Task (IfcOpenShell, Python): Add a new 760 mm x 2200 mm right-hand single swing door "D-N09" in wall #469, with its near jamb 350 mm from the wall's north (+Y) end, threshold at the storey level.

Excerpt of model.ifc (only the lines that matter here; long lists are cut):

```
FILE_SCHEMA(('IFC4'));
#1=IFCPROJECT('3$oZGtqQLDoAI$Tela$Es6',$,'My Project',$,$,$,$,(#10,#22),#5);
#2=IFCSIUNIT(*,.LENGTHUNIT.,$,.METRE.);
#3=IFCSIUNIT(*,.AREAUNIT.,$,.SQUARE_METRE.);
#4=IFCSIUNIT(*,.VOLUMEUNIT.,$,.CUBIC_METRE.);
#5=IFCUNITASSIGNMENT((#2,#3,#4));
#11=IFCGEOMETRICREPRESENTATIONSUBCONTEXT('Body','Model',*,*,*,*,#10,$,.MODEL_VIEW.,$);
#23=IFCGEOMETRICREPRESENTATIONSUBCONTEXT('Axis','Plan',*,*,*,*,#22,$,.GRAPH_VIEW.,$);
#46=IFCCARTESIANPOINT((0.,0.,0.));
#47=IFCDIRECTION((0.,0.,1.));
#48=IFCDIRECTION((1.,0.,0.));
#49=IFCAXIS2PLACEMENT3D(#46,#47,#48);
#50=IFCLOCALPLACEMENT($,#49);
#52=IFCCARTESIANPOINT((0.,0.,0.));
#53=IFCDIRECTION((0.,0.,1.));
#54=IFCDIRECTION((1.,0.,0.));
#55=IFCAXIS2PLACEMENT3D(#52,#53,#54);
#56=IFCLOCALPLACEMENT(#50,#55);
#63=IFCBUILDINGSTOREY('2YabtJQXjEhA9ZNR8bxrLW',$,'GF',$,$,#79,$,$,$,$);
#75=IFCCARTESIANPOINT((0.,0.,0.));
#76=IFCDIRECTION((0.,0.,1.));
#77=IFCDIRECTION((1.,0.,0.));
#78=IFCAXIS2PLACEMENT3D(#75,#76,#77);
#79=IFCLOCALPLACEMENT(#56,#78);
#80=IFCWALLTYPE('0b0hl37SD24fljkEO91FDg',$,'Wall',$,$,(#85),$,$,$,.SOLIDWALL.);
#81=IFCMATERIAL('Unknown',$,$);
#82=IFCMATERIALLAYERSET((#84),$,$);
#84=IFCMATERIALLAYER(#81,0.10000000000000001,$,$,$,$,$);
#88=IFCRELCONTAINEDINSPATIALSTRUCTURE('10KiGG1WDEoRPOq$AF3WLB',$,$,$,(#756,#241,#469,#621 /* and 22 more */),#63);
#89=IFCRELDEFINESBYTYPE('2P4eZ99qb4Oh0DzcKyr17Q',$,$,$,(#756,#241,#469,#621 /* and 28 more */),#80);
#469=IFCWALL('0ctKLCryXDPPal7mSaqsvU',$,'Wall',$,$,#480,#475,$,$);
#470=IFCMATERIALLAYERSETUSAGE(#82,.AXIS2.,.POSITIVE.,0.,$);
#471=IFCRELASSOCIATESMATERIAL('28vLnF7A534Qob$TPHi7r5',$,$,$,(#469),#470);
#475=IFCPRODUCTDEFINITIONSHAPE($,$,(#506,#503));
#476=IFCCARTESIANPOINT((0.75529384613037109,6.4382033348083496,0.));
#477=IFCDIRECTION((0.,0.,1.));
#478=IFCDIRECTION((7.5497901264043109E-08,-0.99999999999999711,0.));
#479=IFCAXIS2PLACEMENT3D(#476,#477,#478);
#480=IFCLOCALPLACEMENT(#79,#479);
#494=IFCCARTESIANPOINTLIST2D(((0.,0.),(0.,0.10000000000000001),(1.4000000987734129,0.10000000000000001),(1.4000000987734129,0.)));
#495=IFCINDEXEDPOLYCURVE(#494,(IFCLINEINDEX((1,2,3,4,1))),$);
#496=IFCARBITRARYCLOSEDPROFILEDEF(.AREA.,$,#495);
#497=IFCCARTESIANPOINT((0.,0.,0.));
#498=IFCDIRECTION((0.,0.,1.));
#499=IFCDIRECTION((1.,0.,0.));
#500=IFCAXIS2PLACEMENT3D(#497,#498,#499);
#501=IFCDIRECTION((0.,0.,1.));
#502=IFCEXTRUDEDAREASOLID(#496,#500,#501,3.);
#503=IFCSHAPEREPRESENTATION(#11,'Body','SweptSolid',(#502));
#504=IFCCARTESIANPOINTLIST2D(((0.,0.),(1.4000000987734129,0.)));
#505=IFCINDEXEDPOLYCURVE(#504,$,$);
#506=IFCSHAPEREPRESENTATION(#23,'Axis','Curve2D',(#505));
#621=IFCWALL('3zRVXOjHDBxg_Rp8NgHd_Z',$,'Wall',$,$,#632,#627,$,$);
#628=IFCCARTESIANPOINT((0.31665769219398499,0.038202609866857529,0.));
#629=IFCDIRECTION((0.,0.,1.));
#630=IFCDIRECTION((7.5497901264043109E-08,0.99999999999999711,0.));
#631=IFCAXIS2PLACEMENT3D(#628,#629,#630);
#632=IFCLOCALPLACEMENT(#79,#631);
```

```python
import numpy as np
import ifcopenshell
import ifcopenshell.api.feature
import ifcopenshell.api.geometry
import ifcopenshell.api.root
import ifcopenshell.api.spatial
import ifcopenshell.geom
import ifcopenshell.util.element
import ifcopenshell.util.placement
import ifcopenshell.util.representation
import ifcopenshell.util.shape
import ifcopenshell.util.unit

model = ifcopenshell.open("model.ifc")
unit_scale = ifcopenshell.util.unit.calculate_unit_scale(model)
settings = ifcopenshell.geom.settings()


def volume(element):
    """Net volume in cubic metres, openings subtracted."""
    shape = ifcopenshell.geom.create_shape(settings, element)
    return ifcopenshell.util.shape.get_volume(shape.geometry)


wall = model.by_guid("0ctKLCryXDPPal7mSaqsvU")
storey = ifcopenshell.util.element.get_container(wall, ifc_class="IfcBuildingStorey")
context = ifcopenshell.util.representation.get_context(model, "Model", "Body", "MODEL_VIEW")
before = volume(wall)

width, height, from_end, sill = 0.76, 2.2, 0.35, 0.0  # metres

# The wall runs along its own X axis, and the end named is its -X end.
wall_shape = ifcopenshell.geom.create_shape(settings, wall)
x, y, z = ifcopenshell.util.shape.get_vertices(wall_shape.geometry).T
start = x.min() + from_end
face, thickness = float(y.min()), float(y.max() - y.min())
wall_matrix = ifcopenshell.util.placement.get_local_placement(wall.ObjectPlacement)
level = ifcopenshell.util.placement.get_local_placement(storey.ObjectPlacement)[2, 3]


def in_wall(x, y):
    """Placement at x, y metres in the wall's axes, at sill height."""
    matrix = wall_matrix.copy()
    matrix[:, 3] = wall_matrix @ np.array([x / unit_scale, y / unit_scale, 0.0, 1.0])
    matrix[2, 3] = level + sill / unit_scale
    return matrix


# Opening: a box that overshoots both wall faces by 50 mm.
opening = ifcopenshell.api.root.create_entity(model, ifc_class="IfcOpeningElement", predefined_type="OPENING")
box = ifcopenshell.api.geometry.add_wall_representation(
    model, context=context, length=width, height=height, thickness=thickness + 0.1
)
ifcopenshell.api.geometry.assign_representation(model, product=opening, representation=box)
ifcopenshell.api.geometry.edit_object_placement(model, product=opening, matrix=in_wall(start, face - 0.05), is_si=False)
ifcopenshell.api.feature.add_feature(model, feature=opening, element=wall)

door = ifcopenshell.api.root.create_entity(model, ifc_class="IfcDoor", name="D-N09", predefined_type="DOOR")
door.OverallWidth, door.OverallHeight = width / unit_scale, height / unit_scale
door.OperationType = "SINGLE_SWING_RIGHT"
body = ifcopenshell.api.geometry.add_door_representation(
    model,
    context=context,
    overall_width=door.OverallWidth,
    overall_height=door.OverallHeight,
    operation_type="SINGLE_SWING_RIGHT",
    lining_properties={"LiningDepth": thickness / unit_scale, "ThresholdDepth": thickness / unit_scale},
)
ifcopenshell.api.geometry.assign_representation(model, product=door, representation=body)
ifcopenshell.api.spatial.assign_container(model, products=[door], relating_structure=storey)
ifcopenshell.api.feature.add_filling(model, opening=opening, element=door)

# The lining spans the wall, so the door starts at the wall face.
ifcopenshell.api.geometry.edit_object_placement(model, product=door, matrix=in_wall(start, face), is_si=False)

after = volume(wall)

print(f"wall volume {before:.3f} -> {after:.3f} m3")

model.write("model-out.ifc")
```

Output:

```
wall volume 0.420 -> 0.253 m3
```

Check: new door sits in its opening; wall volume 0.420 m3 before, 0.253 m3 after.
